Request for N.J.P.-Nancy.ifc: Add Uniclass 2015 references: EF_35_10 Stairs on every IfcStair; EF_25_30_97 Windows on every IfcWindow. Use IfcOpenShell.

First a look at what the model holds.

```python
import ifcopenshell

model = ifcopenshell.open("N.J.P.-Nancy.ifc")
print(model.schema)
print("classifications:", [c.Name for c in model.by_type("IfcClassification")])
for ifc_class in ("IfcDoor", "IfcRoof", "IfcStair", "IfcWall", "IfcWindow"):
    print(ifc_class, len(model.by_type(ifc_class)))
```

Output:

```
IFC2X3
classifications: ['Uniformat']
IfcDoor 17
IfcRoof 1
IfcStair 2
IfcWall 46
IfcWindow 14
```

```python
import ifcopenshell
import ifcopenshell.api.classification

model = ifcopenshell.open("N.J.P.-Nancy.ifc")

# IFC2X3 requires Source and Edition and has no link from the project to the system.
system = model.create_entity("IfcClassification", Source="NBS", Edition="2015", Name="Uniclass 2015")

codes = {
    "IfcStair": ("EF_35_10", "Stairs"),
    "IfcWindow": ("EF_25_30_97", "Windows"),
}
for ifc_class, (code, name) in codes.items():
    products = model.by_type(ifc_class)
    ifcopenshell.api.classification.add_reference(
        model, products=products, classification=system, identification=code, name=name
    )
    print(code, len(products))

model.write("N.J.P.-Nancy_edited.ifc")
```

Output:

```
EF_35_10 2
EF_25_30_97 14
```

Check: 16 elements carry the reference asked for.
